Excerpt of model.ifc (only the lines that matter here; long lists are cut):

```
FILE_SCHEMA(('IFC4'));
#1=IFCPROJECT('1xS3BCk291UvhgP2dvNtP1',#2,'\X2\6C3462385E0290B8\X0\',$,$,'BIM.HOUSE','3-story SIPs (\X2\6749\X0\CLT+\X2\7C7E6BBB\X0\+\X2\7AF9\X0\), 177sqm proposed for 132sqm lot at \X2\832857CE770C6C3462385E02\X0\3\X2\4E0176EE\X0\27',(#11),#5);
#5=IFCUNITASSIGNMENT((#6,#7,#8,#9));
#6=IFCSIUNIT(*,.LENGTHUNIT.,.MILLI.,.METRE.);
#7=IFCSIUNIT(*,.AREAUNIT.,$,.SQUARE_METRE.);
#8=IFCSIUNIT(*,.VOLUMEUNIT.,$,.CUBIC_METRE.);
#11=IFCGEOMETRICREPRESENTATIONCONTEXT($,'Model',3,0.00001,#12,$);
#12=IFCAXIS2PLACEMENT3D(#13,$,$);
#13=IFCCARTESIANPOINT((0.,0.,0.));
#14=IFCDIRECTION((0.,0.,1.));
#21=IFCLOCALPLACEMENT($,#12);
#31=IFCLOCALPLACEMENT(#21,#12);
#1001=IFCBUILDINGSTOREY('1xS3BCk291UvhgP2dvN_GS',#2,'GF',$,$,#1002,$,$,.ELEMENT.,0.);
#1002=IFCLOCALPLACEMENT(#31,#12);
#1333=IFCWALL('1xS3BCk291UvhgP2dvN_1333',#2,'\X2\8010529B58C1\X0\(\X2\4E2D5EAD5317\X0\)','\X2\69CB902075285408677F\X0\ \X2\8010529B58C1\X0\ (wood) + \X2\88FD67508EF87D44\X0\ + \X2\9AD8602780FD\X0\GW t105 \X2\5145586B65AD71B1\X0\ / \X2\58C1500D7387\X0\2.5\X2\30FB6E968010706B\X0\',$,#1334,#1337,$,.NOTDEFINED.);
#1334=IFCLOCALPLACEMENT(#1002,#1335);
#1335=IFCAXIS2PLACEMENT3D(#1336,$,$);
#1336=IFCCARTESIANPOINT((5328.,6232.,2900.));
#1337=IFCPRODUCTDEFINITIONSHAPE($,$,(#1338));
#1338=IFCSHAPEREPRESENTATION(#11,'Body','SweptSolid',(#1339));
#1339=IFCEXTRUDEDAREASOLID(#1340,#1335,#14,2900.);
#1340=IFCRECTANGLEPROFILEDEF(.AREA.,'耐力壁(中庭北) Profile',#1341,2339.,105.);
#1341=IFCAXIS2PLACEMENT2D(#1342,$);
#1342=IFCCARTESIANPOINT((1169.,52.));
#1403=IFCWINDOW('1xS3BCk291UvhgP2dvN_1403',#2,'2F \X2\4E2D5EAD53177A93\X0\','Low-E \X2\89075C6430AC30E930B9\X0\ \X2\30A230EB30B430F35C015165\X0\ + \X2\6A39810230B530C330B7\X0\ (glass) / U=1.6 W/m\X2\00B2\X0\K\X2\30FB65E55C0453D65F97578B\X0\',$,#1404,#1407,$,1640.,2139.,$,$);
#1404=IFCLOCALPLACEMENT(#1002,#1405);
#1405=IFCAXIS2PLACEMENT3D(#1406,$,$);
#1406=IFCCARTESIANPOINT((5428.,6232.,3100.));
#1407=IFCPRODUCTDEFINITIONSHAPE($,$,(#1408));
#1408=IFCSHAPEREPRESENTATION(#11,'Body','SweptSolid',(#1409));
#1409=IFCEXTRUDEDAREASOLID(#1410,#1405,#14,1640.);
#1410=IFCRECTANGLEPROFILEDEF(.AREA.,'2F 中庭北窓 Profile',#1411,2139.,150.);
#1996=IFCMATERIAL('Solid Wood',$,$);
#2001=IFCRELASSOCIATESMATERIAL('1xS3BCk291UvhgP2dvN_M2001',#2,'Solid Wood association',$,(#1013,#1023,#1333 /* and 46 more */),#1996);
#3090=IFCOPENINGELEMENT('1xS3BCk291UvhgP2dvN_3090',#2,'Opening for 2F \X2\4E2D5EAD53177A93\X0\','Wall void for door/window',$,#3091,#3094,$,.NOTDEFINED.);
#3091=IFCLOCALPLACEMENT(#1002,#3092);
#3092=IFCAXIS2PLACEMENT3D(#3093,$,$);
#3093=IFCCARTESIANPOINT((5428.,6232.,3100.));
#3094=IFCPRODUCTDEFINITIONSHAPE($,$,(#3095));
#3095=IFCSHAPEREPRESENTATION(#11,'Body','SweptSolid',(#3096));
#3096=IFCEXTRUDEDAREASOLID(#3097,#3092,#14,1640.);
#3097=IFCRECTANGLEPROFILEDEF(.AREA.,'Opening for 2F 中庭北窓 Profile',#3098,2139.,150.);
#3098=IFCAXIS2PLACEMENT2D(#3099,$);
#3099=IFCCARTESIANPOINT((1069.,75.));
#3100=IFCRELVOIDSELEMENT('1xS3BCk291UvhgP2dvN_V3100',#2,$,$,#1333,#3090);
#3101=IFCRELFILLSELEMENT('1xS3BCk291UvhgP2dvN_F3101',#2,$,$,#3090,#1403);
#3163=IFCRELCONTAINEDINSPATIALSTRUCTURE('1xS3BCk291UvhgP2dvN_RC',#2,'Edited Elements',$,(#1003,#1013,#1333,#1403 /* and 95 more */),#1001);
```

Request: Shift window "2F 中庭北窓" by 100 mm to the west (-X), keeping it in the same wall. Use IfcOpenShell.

```python
import ifcopenshell
import ifcopenshell.api.geometry
import ifcopenshell.util.placement

model = ifcopenshell.open("model.ifc")

window = model.by_id(1403)
opening = window.FillsVoids[0].RelatingOpeningElement
wall = opening.VoidsElements[0].RelatingBuildingElement

wall_matrix = ifcopenshell.util.placement.get_local_placement(wall.ObjectPlacement)
shift = wall_matrix[:3, 0] * -100.0
before = ifcopenshell.util.placement.get_local_placement(window.ObjectPlacement)[:3, 3].copy()

# The window is not placed relative to its opening, so move both.
for product in (opening, window):
    matrix = ifcopenshell.util.placement.get_local_placement(product.ObjectPlacement)
    matrix[:3, 3] += shift
    ifcopenshell.api.geometry.edit_object_placement(model, product=product, matrix=matrix, is_si=False)

after = ifcopenshell.util.placement.get_local_placement(window.ObjectPlacement)[:3, 3]
print("window moved by", (after - before).round(3) + 0.0)

model.write("model_v2.ifc")
```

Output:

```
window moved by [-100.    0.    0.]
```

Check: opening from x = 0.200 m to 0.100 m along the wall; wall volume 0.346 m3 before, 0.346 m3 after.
